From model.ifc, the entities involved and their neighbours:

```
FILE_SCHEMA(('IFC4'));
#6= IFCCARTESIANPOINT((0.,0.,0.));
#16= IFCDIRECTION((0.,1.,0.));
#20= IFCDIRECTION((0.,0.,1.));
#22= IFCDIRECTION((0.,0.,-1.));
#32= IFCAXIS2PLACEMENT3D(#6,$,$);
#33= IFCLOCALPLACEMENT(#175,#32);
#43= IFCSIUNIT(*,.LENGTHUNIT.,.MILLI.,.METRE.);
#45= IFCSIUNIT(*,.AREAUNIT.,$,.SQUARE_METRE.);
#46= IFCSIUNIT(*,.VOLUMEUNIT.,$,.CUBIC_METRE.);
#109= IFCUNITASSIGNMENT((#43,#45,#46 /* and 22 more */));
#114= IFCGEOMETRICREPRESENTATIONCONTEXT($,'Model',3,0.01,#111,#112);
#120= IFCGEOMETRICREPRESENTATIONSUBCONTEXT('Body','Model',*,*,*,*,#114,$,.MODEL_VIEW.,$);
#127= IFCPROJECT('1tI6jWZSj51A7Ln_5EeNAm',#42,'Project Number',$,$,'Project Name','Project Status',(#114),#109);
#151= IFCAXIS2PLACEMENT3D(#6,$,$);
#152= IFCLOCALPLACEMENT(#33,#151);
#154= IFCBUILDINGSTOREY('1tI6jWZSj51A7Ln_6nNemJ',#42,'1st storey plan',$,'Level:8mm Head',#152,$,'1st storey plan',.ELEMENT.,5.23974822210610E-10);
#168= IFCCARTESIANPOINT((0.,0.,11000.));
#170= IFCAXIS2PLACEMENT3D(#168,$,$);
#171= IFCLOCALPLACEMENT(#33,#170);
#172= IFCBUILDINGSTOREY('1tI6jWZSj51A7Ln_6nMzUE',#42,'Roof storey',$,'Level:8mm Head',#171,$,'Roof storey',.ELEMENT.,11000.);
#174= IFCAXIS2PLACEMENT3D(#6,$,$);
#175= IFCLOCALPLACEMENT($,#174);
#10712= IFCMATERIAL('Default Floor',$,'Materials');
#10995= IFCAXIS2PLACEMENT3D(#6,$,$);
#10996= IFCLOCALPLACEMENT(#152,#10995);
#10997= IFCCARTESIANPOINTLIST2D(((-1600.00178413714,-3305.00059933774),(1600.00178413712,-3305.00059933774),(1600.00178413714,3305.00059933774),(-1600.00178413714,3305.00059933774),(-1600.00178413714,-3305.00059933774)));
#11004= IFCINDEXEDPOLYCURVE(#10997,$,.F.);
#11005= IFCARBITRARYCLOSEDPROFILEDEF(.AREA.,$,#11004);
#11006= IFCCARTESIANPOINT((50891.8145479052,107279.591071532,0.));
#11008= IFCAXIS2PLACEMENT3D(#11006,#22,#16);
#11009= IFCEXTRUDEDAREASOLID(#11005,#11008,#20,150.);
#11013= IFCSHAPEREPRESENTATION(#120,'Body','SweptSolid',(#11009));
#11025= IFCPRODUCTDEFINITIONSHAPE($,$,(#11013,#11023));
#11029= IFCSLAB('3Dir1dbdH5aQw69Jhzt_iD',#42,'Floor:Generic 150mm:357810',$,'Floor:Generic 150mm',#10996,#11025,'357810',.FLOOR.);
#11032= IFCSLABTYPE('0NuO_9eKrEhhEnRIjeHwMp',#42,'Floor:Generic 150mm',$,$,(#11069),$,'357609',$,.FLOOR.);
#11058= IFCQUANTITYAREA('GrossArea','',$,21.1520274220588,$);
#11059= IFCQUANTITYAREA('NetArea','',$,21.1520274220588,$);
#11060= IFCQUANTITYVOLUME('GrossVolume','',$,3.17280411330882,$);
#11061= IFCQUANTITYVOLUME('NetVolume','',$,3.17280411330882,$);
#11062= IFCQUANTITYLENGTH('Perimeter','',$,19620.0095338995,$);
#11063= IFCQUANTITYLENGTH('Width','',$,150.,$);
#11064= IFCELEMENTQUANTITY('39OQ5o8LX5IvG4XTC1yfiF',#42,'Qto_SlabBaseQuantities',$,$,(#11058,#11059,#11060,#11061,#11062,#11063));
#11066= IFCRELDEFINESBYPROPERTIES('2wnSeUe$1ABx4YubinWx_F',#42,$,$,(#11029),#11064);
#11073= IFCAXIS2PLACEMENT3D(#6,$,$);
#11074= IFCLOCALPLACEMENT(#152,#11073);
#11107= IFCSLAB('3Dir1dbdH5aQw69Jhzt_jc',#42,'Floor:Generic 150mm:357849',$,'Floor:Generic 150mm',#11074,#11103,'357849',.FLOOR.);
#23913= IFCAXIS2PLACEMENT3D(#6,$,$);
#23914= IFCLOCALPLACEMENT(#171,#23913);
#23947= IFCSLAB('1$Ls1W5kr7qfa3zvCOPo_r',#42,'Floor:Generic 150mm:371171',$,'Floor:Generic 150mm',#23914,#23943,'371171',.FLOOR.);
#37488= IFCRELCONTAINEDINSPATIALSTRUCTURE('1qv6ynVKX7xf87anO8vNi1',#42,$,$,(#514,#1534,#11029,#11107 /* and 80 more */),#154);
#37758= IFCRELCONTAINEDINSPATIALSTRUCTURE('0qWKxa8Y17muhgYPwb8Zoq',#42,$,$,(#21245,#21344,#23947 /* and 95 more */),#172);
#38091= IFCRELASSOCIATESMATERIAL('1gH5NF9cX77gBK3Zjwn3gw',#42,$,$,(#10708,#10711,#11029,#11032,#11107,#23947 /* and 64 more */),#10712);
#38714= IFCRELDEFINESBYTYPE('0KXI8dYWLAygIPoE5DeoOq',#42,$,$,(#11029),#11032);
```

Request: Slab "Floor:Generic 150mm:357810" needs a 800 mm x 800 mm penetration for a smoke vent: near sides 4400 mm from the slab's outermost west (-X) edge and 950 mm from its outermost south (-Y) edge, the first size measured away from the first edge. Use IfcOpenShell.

```python
import numpy as np
import ifcopenshell
import ifcopenshell.api.feature
import ifcopenshell.api.geometry
import ifcopenshell.api.pset
import ifcopenshell.api.root
import ifcopenshell.geom
import ifcopenshell.util.element
import ifcopenshell.util.placement
import ifcopenshell.util.representation
import ifcopenshell.util.shape
import ifcopenshell.util.unit

model = ifcopenshell.open("model.ifc")
unit_scale = ifcopenshell.util.unit.calculate_unit_scale(model)
area_scale = ifcopenshell.util.unit.calculate_unit_scale(model, "AREAUNIT")
volume_scale = ifcopenshell.util.unit.calculate_unit_scale(model, "VOLUMEUNIT")
settings = ifcopenshell.geom.settings()


def volume(element):
    """Net volume in cubic metres, openings subtracted."""
    shape = ifcopenshell.geom.create_shape(settings, element)
    return ifcopenshell.util.shape.get_volume(shape.geometry)


slab = model.by_guid("3Dir1dbdH5aQw69Jhzt_iD")
before = volume(slab)

# Extent in the slab's own axes, in metres. The edges named are its -X and -Y sides.
slab_shape = ifcopenshell.geom.create_shape(settings, slab)
vertices = ifcopenshell.util.shape.get_vertices(slab_shape.geometry)
x_min, y_min, bottom = vertices.min(axis=0)
top = vertices[:, 2].max()

opening = ifcopenshell.api.root.create_entity(model, ifc_class="IfcOpeningElement", name="Smoke vent opening", predefined_type="OPENING")
context = ifcopenshell.util.representation.get_context(model, "Model", "Body", "MODEL_VIEW")
width, depth = 0.8, 0.8
outline = [(0.0, 0.0), (width, 0.0), (width, depth), (0.0, depth), (0.0, 0.0)]
# Overshoot both faces by 50 mm so the cut is clean.
shape = ifcopenshell.api.geometry.add_slab_representation(
    model, context=context, depth=top - bottom + 0.1, polyline=outline
)
ifcopenshell.api.geometry.assign_representation(model, product=opening, representation=shape)

matrix = ifcopenshell.util.placement.get_local_placement(slab.ObjectPlacement)
matrix[:, 3] = matrix @ np.append(np.array([x_min + 4.4, y_min + 0.95, bottom - 0.05]) / unit_scale, 1.0)
ifcopenshell.api.geometry.edit_object_placement(model, product=opening, matrix=matrix, is_si=False)
ifcopenshell.api.feature.add_feature(model, feature=opening, element=slab)

after = volume(slab)

# Update the slab's stored quantities.
qto = model.by_id(ifcopenshell.util.element.get_pset(slab, "Qto_SlabBaseQuantities", should_inherit=False)["id"])
ifcopenshell.api.pset.edit_qto(model, qto=qto, properties={
    "NetArea": after / (top - bottom) / area_scale,
    "NetVolume": after / volume_scale,
})

print(f"slab volume {before:.3f} -> {after:.3f} m3")

model.write("model_edited.ifc")
```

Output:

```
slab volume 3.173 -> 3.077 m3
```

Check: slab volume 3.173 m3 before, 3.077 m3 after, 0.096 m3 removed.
